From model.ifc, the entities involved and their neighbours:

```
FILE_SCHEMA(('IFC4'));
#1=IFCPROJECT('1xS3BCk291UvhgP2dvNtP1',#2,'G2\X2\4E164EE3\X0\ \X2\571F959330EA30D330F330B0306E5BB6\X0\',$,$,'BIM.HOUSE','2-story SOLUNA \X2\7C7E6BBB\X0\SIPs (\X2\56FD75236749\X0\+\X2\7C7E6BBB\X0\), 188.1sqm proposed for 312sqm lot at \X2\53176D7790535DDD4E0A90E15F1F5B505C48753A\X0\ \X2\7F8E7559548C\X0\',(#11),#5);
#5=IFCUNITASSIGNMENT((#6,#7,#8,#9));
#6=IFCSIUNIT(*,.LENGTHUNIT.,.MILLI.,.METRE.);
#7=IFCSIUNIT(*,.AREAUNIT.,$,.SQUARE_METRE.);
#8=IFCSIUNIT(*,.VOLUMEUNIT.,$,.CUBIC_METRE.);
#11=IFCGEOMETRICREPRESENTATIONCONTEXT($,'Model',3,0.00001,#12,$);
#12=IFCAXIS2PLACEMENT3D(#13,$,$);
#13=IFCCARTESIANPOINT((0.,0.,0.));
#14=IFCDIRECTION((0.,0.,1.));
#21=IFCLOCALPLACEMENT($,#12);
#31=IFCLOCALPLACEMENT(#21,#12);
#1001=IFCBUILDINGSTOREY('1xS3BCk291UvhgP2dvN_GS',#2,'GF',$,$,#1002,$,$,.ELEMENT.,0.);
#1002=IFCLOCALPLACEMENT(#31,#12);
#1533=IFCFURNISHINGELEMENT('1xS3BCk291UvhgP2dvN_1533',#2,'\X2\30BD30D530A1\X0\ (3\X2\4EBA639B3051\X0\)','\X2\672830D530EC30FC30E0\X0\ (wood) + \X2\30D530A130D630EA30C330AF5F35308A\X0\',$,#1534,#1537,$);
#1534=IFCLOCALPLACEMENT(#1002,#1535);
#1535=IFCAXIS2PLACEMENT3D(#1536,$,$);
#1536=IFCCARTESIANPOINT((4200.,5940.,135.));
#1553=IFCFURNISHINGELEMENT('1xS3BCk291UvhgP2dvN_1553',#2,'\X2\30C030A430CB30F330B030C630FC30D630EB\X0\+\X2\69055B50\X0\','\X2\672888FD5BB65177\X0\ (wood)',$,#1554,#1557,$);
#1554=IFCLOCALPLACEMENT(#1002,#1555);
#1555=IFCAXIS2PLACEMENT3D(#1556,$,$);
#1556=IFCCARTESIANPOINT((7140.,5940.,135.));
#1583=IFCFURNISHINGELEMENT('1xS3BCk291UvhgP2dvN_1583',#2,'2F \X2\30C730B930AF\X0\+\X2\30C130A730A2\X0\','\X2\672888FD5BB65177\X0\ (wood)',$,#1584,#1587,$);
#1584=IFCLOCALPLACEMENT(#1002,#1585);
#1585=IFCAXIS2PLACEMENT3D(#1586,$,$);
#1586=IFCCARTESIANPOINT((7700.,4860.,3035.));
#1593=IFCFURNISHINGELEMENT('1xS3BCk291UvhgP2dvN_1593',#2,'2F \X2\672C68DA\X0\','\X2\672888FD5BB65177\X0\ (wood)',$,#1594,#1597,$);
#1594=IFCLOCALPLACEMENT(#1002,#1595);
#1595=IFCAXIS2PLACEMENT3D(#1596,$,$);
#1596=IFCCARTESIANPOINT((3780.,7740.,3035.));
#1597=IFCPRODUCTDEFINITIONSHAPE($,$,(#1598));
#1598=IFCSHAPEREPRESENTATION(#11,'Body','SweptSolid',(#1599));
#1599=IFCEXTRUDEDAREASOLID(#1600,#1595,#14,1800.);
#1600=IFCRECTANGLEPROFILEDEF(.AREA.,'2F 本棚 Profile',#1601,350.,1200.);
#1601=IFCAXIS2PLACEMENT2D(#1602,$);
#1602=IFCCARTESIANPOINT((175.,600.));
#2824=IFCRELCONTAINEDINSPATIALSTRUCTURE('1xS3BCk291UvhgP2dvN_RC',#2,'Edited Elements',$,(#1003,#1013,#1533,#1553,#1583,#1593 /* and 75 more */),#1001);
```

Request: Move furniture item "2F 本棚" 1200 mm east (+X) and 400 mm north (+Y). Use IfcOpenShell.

```python
import ifcopenshell
import ifcopenshell.api.geometry
import ifcopenshell.util.placement
import ifcopenshell.util.unit

model = ifcopenshell.open("model.ifc")
unit_scale = ifcopenshell.util.unit.calculate_unit_scale(model)

item = model.by_id(1593)
matrix = ifcopenshell.util.placement.get_local_placement(item.ObjectPlacement)
matrix[0, 3] += 1.2 / unit_scale
matrix[1, 3] += 0.4 / unit_scale
ifcopenshell.api.geometry.edit_object_placement(model, product=item, matrix=matrix, is_si=False)

print(ifcopenshell.util.placement.get_local_placement(item.ObjectPlacement).round(3) + 0.0)

model.write("model_v2.ifc")
```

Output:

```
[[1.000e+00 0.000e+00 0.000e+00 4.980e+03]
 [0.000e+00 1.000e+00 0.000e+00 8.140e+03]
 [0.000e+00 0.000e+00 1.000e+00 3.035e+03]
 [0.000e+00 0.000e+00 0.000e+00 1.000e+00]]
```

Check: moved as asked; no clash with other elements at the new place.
